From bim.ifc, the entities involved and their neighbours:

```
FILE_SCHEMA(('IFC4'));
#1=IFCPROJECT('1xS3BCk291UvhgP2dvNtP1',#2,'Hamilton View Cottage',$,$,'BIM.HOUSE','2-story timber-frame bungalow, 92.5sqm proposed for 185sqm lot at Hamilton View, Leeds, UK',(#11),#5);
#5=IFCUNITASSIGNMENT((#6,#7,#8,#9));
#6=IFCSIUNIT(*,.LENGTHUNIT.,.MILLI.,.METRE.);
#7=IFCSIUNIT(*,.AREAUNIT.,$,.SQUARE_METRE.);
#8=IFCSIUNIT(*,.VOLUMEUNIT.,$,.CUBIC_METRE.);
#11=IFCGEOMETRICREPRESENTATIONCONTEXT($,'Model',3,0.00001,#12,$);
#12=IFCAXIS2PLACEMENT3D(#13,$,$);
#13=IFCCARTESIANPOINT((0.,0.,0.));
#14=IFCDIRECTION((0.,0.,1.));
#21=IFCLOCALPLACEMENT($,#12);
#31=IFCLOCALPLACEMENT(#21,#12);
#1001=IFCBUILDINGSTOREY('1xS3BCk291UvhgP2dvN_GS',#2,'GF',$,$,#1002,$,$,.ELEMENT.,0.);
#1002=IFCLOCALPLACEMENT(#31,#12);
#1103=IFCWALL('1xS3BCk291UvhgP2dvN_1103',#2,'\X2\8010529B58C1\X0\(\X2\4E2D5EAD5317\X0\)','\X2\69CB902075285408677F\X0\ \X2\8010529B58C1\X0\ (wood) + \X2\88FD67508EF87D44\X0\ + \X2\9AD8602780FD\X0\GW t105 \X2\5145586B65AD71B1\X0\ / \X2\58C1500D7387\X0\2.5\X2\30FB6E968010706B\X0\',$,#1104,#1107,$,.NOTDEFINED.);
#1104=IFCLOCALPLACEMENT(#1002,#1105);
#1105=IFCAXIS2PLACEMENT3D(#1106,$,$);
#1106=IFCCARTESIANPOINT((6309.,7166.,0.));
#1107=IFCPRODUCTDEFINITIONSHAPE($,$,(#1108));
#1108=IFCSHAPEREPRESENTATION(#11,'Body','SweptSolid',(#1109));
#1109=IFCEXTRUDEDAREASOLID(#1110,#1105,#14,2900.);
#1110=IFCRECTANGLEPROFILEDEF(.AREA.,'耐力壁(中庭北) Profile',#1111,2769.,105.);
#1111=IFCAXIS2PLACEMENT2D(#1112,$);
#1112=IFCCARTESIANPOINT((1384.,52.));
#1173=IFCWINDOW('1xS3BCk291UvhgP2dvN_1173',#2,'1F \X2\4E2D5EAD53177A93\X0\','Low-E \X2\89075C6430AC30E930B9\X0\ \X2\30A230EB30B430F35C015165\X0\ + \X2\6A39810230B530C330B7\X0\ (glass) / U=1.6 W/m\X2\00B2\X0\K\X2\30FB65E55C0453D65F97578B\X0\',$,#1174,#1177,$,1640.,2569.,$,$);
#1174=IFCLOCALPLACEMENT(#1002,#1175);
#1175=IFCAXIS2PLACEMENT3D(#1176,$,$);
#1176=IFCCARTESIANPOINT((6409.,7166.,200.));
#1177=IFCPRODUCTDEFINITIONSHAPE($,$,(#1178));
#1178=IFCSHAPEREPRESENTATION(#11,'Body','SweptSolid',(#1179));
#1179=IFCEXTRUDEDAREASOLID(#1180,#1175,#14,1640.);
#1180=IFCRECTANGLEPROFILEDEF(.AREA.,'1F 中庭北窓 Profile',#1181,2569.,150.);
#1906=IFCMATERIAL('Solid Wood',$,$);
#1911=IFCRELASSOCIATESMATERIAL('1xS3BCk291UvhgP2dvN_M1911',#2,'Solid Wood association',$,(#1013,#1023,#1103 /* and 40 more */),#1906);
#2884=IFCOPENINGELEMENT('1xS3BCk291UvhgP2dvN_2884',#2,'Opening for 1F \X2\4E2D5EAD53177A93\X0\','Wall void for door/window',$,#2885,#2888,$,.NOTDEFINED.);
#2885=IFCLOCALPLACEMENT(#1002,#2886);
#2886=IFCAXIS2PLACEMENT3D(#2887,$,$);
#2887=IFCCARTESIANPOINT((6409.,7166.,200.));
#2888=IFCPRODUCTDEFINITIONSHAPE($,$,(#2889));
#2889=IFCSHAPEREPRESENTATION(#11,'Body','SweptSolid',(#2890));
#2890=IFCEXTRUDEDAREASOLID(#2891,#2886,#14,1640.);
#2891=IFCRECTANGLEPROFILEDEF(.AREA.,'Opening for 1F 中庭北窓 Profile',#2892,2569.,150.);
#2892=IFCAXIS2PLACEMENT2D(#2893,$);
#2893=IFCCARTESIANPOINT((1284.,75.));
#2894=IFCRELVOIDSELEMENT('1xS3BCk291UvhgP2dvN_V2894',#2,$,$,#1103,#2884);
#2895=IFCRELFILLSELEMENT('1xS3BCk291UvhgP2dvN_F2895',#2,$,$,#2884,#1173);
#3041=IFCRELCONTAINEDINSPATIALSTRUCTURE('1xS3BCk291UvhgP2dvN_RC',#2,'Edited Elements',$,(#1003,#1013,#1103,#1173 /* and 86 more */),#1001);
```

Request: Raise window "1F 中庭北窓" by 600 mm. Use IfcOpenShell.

```python
import numpy as np
import ifcopenshell
import ifcopenshell.api.geometry
import ifcopenshell.util.placement
import ifcopenshell.util.unit

model = ifcopenshell.open("bim.ifc")
unit_scale = ifcopenshell.util.unit.calculate_unit_scale(model)

window = model.by_guid("1xS3BCk291UvhgP2dvN_1173")
opening = window.FillsVoids[0].RelatingOpeningElement
dz = 600.0

shift = np.array([0.0, 0.0, dz])
# The window is not placed relative to its opening, so move both.
for product in (opening, window):
    matrix = ifcopenshell.util.placement.get_local_placement(product.ObjectPlacement)
    matrix[:3, 3] += shift
    ifcopenshell.api.geometry.edit_object_placement(model, product=product, matrix=matrix, is_si=False)

print(f"moved by {dz * unit_scale:+.3f} m")

model.write("bim_edited.ifc")
```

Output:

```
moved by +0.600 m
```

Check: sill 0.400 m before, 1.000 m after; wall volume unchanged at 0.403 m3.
